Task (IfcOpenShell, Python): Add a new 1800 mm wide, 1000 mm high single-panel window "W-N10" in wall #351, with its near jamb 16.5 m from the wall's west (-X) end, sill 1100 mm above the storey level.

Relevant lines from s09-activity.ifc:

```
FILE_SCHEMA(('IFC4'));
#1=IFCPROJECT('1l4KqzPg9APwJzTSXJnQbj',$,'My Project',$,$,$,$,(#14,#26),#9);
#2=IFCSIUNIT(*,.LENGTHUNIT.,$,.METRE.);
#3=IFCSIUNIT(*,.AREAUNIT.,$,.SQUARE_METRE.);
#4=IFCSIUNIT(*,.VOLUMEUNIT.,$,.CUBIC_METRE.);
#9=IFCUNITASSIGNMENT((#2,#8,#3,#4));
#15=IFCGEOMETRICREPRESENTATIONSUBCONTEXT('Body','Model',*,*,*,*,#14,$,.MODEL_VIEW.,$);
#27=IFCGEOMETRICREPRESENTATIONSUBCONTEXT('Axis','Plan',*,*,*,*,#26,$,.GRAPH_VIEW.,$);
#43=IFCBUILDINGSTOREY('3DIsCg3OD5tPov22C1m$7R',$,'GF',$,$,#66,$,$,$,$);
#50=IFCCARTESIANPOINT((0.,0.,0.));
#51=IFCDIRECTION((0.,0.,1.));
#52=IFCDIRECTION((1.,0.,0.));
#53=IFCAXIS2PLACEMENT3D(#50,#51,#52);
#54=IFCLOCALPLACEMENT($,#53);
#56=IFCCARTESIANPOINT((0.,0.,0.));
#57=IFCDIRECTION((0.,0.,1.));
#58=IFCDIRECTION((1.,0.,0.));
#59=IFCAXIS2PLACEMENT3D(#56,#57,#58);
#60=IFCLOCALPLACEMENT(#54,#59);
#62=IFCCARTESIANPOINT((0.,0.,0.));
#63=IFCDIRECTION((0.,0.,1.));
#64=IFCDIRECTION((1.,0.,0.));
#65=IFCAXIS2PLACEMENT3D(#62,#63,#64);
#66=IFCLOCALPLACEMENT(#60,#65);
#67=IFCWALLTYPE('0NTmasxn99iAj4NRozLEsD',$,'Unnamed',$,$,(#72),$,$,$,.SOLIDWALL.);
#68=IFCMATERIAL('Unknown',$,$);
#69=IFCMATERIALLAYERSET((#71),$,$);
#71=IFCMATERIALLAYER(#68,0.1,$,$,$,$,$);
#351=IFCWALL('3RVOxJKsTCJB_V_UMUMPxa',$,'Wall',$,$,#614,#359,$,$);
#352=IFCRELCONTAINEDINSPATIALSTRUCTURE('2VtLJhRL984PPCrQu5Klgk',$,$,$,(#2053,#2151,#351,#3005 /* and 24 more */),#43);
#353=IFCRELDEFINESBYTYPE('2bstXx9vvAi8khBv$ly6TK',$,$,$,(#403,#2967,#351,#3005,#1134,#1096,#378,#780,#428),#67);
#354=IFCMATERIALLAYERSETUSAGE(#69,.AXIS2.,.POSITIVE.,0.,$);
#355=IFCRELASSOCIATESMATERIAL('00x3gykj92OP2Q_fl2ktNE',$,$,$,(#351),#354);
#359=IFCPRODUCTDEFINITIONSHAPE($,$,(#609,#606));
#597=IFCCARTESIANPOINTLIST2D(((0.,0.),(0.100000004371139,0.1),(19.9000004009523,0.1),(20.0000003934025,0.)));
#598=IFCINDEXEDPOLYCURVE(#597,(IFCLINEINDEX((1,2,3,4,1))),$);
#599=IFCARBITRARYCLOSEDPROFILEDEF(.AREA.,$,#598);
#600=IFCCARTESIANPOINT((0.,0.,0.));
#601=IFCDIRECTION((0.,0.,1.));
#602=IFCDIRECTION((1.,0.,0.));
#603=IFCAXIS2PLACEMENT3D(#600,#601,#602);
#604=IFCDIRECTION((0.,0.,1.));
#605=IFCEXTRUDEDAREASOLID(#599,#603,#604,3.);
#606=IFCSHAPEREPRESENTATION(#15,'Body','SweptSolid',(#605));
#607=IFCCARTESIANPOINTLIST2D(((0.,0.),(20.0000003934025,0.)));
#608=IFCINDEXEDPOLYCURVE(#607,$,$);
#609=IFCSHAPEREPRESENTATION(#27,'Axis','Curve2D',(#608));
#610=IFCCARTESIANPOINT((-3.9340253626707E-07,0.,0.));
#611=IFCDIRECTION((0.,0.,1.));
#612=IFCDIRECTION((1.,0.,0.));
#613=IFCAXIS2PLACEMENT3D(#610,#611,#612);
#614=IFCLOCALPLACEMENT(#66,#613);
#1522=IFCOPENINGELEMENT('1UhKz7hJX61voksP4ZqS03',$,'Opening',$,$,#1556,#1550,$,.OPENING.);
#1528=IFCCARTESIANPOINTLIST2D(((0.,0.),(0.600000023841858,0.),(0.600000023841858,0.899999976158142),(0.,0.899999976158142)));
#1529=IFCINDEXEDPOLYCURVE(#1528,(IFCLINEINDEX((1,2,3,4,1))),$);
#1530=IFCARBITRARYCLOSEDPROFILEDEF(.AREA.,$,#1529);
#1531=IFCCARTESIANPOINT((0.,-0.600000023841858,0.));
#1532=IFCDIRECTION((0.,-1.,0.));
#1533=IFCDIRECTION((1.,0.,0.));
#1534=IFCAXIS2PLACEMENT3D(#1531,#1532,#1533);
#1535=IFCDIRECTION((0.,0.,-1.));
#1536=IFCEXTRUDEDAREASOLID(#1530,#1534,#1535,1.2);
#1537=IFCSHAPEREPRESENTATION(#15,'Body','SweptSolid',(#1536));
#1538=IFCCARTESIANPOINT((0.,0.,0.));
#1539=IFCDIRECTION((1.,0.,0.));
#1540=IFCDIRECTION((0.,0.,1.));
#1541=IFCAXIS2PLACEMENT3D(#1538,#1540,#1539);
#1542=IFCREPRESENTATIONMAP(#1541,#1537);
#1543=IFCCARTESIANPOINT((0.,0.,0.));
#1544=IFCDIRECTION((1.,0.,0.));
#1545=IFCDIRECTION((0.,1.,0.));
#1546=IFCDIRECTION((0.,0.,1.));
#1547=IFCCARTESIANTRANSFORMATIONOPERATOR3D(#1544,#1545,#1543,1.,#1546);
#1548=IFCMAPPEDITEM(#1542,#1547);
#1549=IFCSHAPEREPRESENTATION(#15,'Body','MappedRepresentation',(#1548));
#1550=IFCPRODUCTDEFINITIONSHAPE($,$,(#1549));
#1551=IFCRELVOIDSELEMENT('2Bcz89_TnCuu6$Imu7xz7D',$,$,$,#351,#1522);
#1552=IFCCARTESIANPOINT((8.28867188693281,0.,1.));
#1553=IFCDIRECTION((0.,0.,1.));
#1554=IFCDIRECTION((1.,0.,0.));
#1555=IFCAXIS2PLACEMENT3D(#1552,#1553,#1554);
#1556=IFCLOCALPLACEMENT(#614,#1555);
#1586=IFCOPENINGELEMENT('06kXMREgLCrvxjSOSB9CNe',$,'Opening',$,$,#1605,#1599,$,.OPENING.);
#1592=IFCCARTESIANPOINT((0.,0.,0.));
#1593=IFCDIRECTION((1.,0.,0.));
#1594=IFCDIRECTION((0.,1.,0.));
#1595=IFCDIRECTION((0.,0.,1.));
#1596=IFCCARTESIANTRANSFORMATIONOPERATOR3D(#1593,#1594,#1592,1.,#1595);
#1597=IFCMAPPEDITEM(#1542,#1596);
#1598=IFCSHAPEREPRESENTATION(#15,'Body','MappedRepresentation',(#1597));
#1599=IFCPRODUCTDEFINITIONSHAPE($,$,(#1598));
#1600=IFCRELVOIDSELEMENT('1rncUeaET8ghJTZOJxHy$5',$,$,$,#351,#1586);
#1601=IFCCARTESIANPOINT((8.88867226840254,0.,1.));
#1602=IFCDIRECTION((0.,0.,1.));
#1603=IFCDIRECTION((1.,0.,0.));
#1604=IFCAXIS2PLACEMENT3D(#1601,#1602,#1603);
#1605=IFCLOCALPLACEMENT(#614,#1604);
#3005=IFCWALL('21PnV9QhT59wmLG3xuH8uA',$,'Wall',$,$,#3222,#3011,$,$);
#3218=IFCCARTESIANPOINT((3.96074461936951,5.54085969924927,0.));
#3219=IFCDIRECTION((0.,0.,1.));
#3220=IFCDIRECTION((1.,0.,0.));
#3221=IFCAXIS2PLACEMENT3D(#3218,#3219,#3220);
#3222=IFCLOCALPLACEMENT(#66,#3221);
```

```python
import numpy as np
import ifcopenshell
import ifcopenshell.api.feature
import ifcopenshell.api.geometry
import ifcopenshell.api.root
import ifcopenshell.api.spatial
import ifcopenshell.geom
import ifcopenshell.util.element
import ifcopenshell.util.placement
import ifcopenshell.util.representation
import ifcopenshell.util.shape
import ifcopenshell.util.unit

model = ifcopenshell.open("s09-activity.ifc")
unit_scale = ifcopenshell.util.unit.calculate_unit_scale(model)
settings = ifcopenshell.geom.settings()


def volume(element):
    """Net volume in cubic metres, openings subtracted."""
    shape = ifcopenshell.geom.create_shape(settings, element)
    return ifcopenshell.util.shape.get_volume(shape.geometry)


wall = model.by_id(351)
storey = ifcopenshell.util.element.get_container(wall, ifc_class="IfcBuildingStorey")
context = ifcopenshell.util.representation.get_context(model, "Model", "Body", "MODEL_VIEW")
before = volume(wall)

width, height, from_end, sill = 1.8, 1, 16.5, 1.1  # metres

# The wall runs along its own X axis, and the end named is its -X end.
wall_shape = ifcopenshell.geom.create_shape(settings, wall)
x, y, z = ifcopenshell.util.shape.get_vertices(wall_shape.geometry).T
start = x.min() + from_end
face, thickness = float(y.min()), float(y.max() - y.min())
wall_matrix = ifcopenshell.util.placement.get_local_placement(wall.ObjectPlacement)
level = ifcopenshell.util.placement.get_local_placement(storey.ObjectPlacement)[2, 3]


def in_wall(x, y):
    """Placement at x, y metres in the wall's axes, at sill height."""
    matrix = wall_matrix.copy()
    matrix[:, 3] = wall_matrix @ np.array([x / unit_scale, y / unit_scale, 0.0, 1.0])
    matrix[2, 3] = level + sill / unit_scale
    return matrix


# Opening: a box that overshoots both wall faces by 50 mm.
opening = ifcopenshell.api.root.create_entity(model, ifc_class="IfcOpeningElement", predefined_type="OPENING")
box = ifcopenshell.api.geometry.add_wall_representation(
    model, context=context, length=width, height=height, thickness=thickness + 0.1
)
ifcopenshell.api.geometry.assign_representation(model, product=opening, representation=box)
ifcopenshell.api.geometry.edit_object_placement(model, product=opening, matrix=in_wall(start, face - 0.05), is_si=False)
ifcopenshell.api.feature.add_feature(model, feature=opening, element=wall)

window = ifcopenshell.api.root.create_entity(model, ifc_class="IfcWindow", name="W-N10", predefined_type="WINDOW")
window.OverallWidth, window.OverallHeight = width / unit_scale, height / unit_scale
window.PartitioningType = "SINGLE_PANEL"
body = ifcopenshell.api.geometry.add_window_representation(
    model,
    context=context,
    overall_width=window.OverallWidth,
    overall_height=window.OverallHeight,
    partition_type="SINGLE_PANEL",
)
ifcopenshell.api.geometry.assign_representation(model, product=window, representation=body)
ifcopenshell.api.spatial.assign_container(model, products=[window], relating_structure=storey)
ifcopenshell.api.feature.add_filling(model, opening=opening, element=window)

# Centre the window in the wall's thickness.
ifcopenshell.api.geometry.edit_object_placement(model, product=window, matrix=in_wall(start, face), is_si=False)
window_shape = ifcopenshell.geom.create_shape(settings, window)
depth = ifcopenshell.util.shape.get_vertices(window_shape.geometry)[:, 1]
offset = face + thickness / 2 - (depth.min() + depth.max()) / 2
ifcopenshell.api.geometry.edit_object_placement(model, product=window, matrix=in_wall(start, offset), is_si=False)

after = volume(wall)

print(f"wall volume {before:.3f} -> {after:.3f} m3")

model.write("s09-activity_v2.ifc")
```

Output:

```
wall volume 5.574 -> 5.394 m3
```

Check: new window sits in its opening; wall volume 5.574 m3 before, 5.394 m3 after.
